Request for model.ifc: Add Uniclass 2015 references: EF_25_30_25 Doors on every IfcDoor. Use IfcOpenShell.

First a look at what the model holds.

```python
import ifcopenshell

model = ifcopenshell.open("model.ifc")
print(model.schema)
print("classifications:", [c.Name for c in model.by_type("IfcClassification")])
for ifc_class in ("IfcDoor", "IfcRoof", "IfcStair", "IfcWall", "IfcWindow"):
    print(ifc_class, len(model.by_type(ifc_class)))
```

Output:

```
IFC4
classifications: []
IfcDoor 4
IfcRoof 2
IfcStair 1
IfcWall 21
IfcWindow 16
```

```python
import ifcopenshell
import ifcopenshell.api.classification

model = ifcopenshell.open("model.ifc")

system = ifcopenshell.api.classification.add_classification(model, classification="Uniclass 2015")

codes = {
    "IfcDoor": ("EF_25_30_25", "Doors"),
}
for ifc_class, (code, name) in codes.items():
    products = model.by_type(ifc_class)
    ifcopenshell.api.classification.add_reference(
        model, products=products, classification=system, identification=code, name=name
    )
    print(code, len(products))

model.write("model-out.ifc")
```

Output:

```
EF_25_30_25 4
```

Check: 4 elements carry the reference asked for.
